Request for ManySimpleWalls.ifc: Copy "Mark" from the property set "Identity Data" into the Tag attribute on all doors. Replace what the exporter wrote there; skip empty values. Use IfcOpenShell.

First a look at what the model holds.

```python
import ifcopenshell
import ifcopenshell.util.element

model = ifcopenshell.open("ManySimpleWalls.ifc")
print(model.schema)
doors = model.by_type("IfcDoor")
print(len(doors), "doors")
for e in doors[:8]:
    source = ifcopenshell.util.element.get_pset(e, "Identity Data", "Mark")
    target = e.Tag
    print(e.id(), repr(source), repr(target), sep=" | ")
```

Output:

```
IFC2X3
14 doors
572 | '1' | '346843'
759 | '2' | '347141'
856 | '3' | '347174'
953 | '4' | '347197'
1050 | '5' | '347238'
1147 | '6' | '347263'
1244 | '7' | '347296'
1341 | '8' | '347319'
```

```python
import ifcopenshell
import ifcopenshell.util.element

model = ifcopenshell.open("ManySimpleWalls.ifc")

count = 0
for e in model.by_type("IfcDoor"):
    value = ifcopenshell.util.element.get_pset(e, "Identity Data", "Mark")
    current = e.Tag
    if not value or not value.strip() or current == value:
        continue
    e.Tag = value
    count += 1

print(count, "doors updated")

model.write("ManySimpleWalls-out.ifc")
```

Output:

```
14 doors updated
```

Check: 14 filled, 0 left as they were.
